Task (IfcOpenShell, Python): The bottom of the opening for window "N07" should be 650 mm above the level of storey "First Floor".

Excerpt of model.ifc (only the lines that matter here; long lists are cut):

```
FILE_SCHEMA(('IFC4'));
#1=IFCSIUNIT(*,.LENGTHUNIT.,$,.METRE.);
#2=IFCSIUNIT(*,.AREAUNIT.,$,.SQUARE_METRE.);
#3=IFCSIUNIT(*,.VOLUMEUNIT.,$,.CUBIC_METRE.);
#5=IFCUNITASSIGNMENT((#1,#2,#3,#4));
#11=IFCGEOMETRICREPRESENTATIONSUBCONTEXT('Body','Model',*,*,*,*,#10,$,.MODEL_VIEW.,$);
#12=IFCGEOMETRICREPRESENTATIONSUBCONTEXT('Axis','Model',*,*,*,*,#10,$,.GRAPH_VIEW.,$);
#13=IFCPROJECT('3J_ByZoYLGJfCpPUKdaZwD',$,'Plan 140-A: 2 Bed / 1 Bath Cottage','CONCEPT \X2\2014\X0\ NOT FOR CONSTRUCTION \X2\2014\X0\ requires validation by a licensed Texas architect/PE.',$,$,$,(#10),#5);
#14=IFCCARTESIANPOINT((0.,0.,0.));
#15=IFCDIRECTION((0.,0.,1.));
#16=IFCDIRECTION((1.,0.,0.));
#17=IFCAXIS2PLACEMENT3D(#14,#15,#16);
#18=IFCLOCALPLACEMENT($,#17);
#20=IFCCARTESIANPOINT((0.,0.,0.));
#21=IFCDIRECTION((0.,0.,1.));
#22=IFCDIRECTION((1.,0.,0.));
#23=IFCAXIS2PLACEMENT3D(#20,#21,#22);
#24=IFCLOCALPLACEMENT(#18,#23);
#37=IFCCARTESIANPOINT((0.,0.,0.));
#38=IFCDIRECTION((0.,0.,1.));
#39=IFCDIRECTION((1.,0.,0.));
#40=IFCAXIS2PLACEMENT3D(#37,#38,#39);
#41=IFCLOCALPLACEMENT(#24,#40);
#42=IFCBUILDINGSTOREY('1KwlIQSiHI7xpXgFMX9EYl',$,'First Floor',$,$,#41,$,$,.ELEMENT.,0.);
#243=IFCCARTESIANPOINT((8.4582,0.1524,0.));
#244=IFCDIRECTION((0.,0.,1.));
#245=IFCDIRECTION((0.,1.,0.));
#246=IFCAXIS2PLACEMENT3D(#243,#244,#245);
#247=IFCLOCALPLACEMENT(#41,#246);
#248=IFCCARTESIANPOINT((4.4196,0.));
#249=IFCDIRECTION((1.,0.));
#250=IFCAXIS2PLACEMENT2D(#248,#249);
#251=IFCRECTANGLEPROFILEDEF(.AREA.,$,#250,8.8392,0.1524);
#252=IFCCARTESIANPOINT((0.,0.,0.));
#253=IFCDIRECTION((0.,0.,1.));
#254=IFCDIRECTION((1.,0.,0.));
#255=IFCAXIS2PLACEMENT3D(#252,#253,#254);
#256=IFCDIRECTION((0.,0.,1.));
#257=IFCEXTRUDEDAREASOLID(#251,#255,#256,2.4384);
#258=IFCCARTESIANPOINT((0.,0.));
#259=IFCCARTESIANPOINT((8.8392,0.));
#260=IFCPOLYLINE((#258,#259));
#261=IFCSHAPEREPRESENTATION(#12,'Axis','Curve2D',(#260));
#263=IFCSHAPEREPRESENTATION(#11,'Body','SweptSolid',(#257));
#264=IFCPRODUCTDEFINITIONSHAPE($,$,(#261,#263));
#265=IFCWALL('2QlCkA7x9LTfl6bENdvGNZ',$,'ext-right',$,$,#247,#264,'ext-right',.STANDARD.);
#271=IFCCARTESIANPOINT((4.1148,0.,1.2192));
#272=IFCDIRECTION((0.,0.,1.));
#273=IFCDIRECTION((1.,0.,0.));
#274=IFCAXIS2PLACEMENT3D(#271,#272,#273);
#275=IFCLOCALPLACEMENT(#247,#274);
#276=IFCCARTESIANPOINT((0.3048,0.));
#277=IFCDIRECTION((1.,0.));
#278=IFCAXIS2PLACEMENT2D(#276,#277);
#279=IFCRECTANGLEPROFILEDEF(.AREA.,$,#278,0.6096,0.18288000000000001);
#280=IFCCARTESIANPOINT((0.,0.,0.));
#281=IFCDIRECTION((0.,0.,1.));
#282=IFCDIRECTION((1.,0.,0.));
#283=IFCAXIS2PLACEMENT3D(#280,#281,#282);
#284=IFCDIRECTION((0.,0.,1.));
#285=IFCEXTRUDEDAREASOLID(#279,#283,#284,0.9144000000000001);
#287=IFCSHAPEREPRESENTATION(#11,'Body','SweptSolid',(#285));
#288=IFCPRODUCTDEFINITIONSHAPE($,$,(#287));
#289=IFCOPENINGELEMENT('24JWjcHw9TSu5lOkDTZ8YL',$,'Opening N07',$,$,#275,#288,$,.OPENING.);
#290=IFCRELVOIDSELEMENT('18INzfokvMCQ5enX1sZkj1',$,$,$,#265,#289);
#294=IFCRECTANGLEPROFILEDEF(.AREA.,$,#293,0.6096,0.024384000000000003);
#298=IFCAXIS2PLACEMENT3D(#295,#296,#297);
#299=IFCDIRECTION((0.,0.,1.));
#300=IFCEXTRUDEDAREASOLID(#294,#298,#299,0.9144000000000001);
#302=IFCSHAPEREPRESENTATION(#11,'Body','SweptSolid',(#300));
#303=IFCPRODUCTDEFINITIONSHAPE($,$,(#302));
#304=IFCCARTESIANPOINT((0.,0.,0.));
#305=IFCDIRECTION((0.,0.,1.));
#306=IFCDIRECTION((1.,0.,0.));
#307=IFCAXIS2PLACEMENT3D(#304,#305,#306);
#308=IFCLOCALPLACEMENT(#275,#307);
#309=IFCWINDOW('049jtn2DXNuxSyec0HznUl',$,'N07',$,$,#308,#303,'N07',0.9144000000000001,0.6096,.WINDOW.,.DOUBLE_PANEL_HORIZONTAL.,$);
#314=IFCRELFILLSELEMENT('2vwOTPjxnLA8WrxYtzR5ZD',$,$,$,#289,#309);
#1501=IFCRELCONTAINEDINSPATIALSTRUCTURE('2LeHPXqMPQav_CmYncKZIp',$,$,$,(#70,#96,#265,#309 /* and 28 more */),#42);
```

```python
import numpy as np
import ifcopenshell
import ifcopenshell.api.geometry
import ifcopenshell.geom
import ifcopenshell.util.element
import ifcopenshell.util.placement
import ifcopenshell.util.shape
import ifcopenshell.util.unit

model = ifcopenshell.open("model.ifc")
unit_scale = ifcopenshell.util.unit.calculate_unit_scale(model)

window = model.by_guid("049jtn2DXNuxSyec0HznUl")
opening = window.FillsVoids[0].RelatingOpeningElement
storey = ifcopenshell.util.element.get_container(window, ifc_class="IfcBuildingStorey")
level = ifcopenshell.util.placement.get_local_placement(storey.ObjectPlacement)[2, 3]

# The opening's origin need not be at the sill, so measure its lowest point.
shape = ifcopenshell.geom.create_shape(ifcopenshell.geom.settings(), opening)
bottom = ifcopenshell.util.shape.get_shape_bottom_elevation(shape, shape.geometry) / unit_scale
dz = level + 0.65 / unit_scale - bottom

shift = np.array([0.0, 0.0, dz])
# The window is placed relative to its opening, so it follows when the opening moves.
matrix = ifcopenshell.util.placement.get_local_placement(opening.ObjectPlacement)
matrix[:3, 3] += shift
ifcopenshell.api.geometry.edit_object_placement(
    model, product=opening, matrix=matrix, is_si=False, should_transform_children=True
)

print(f"moved by {dz * unit_scale:+.3f} m")

model.write("model_updated.ifc")
```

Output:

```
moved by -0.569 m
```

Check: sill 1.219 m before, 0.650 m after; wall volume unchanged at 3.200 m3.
